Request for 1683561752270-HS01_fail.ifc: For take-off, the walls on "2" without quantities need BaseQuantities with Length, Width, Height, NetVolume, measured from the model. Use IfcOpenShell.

First a look at what the model holds.

```python
import ifcopenshell
import ifcopenshell.util.element
import ifcopenshell.util.unit

model = ifcopenshell.open("1683561752270-HS01_fail.ifc")
print(model.schema)
for unit_type in ("LENGTHUNIT", "AREAUNIT", "VOLUMEUNIT"):
    print(unit_type, ifcopenshell.util.unit.calculate_unit_scale(model, unit_type))
storey = next(s for s in model.by_type("IfcBuildingStorey") if s.Name == "2")
walls = [e for e in ifcopenshell.util.element.get_decomposition(storey) if e.is_a("IfcWall")]
for e in sorted(walls, key=lambda e: e.id()):
    print(e.id(), e.is_a(), e.Name, list(ifcopenshell.util.element.get_psets(e, qtos_only=True)), sep=" | ")
```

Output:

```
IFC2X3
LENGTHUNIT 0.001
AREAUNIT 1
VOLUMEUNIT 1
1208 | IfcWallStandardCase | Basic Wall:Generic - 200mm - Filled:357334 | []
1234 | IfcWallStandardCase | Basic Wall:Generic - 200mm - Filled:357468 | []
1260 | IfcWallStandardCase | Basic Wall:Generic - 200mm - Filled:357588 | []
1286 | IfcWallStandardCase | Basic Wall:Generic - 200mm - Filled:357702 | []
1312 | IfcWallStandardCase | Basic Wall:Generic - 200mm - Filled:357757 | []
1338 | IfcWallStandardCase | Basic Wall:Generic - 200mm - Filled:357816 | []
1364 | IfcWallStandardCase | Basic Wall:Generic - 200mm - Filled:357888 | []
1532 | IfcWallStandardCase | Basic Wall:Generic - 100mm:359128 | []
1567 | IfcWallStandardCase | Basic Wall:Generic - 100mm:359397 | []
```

```python
import ifcopenshell
import ifcopenshell.api.pset
import ifcopenshell.geom
import ifcopenshell.util.element
import ifcopenshell.util.shape
import ifcopenshell.util.unit

model = ifcopenshell.open("1683561752270-HS01_fail.ifc")
unit_scale = ifcopenshell.util.unit.calculate_unit_scale(model)
volume_scale = ifcopenshell.util.unit.calculate_unit_scale(model, "VOLUMEUNIT")
settings = ifcopenshell.geom.settings()

storey = next(s for s in model.by_type("IfcBuildingStorey") if s.Name == "2")
walls = [e for e in ifcopenshell.util.element.get_decomposition(storey) if e.is_a("IfcWall")]

for e in sorted(walls, key=lambda e: e.id()):
    if ifcopenshell.util.element.get_psets(e, qtos_only=True, should_inherit=False):
        continue
    # Geometry comes back in metres, in the element's own axes.
    shape = ifcopenshell.geom.create_shape(settings, e)
    values = {
        "Length": ifcopenshell.util.shape.get_x(shape.geometry) / unit_scale,
        "Width": ifcopenshell.util.shape.get_y(shape.geometry) / unit_scale,
        "Height": ifcopenshell.util.shape.get_z(shape.geometry) / unit_scale,
        "NetVolume": ifcopenshell.util.shape.get_volume(shape.geometry) / volume_scale,
    }
    qto = ifcopenshell.api.pset.add_qto(model, product=e, name="BaseQuantities")
    ifcopenshell.api.pset.edit_qto(model, qto=qto, properties=values)
    print(e.id(), {k: round(v, 3) for k, v in values.items()})

model.write("1683561752270-HS01_fail_rev.ifc")
```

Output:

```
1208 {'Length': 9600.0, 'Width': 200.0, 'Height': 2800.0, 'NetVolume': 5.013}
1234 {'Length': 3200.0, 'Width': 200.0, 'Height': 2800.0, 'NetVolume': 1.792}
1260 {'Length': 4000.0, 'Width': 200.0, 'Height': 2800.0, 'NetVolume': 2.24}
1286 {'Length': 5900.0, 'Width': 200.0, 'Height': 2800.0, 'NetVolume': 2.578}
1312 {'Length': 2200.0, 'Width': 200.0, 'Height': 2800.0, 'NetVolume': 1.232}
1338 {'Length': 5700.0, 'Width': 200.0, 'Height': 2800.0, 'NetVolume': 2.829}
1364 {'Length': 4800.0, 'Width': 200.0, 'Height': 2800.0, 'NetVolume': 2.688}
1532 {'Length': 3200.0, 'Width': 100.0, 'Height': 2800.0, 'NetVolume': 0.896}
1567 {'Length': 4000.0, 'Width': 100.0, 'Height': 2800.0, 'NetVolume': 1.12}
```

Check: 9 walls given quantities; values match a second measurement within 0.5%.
